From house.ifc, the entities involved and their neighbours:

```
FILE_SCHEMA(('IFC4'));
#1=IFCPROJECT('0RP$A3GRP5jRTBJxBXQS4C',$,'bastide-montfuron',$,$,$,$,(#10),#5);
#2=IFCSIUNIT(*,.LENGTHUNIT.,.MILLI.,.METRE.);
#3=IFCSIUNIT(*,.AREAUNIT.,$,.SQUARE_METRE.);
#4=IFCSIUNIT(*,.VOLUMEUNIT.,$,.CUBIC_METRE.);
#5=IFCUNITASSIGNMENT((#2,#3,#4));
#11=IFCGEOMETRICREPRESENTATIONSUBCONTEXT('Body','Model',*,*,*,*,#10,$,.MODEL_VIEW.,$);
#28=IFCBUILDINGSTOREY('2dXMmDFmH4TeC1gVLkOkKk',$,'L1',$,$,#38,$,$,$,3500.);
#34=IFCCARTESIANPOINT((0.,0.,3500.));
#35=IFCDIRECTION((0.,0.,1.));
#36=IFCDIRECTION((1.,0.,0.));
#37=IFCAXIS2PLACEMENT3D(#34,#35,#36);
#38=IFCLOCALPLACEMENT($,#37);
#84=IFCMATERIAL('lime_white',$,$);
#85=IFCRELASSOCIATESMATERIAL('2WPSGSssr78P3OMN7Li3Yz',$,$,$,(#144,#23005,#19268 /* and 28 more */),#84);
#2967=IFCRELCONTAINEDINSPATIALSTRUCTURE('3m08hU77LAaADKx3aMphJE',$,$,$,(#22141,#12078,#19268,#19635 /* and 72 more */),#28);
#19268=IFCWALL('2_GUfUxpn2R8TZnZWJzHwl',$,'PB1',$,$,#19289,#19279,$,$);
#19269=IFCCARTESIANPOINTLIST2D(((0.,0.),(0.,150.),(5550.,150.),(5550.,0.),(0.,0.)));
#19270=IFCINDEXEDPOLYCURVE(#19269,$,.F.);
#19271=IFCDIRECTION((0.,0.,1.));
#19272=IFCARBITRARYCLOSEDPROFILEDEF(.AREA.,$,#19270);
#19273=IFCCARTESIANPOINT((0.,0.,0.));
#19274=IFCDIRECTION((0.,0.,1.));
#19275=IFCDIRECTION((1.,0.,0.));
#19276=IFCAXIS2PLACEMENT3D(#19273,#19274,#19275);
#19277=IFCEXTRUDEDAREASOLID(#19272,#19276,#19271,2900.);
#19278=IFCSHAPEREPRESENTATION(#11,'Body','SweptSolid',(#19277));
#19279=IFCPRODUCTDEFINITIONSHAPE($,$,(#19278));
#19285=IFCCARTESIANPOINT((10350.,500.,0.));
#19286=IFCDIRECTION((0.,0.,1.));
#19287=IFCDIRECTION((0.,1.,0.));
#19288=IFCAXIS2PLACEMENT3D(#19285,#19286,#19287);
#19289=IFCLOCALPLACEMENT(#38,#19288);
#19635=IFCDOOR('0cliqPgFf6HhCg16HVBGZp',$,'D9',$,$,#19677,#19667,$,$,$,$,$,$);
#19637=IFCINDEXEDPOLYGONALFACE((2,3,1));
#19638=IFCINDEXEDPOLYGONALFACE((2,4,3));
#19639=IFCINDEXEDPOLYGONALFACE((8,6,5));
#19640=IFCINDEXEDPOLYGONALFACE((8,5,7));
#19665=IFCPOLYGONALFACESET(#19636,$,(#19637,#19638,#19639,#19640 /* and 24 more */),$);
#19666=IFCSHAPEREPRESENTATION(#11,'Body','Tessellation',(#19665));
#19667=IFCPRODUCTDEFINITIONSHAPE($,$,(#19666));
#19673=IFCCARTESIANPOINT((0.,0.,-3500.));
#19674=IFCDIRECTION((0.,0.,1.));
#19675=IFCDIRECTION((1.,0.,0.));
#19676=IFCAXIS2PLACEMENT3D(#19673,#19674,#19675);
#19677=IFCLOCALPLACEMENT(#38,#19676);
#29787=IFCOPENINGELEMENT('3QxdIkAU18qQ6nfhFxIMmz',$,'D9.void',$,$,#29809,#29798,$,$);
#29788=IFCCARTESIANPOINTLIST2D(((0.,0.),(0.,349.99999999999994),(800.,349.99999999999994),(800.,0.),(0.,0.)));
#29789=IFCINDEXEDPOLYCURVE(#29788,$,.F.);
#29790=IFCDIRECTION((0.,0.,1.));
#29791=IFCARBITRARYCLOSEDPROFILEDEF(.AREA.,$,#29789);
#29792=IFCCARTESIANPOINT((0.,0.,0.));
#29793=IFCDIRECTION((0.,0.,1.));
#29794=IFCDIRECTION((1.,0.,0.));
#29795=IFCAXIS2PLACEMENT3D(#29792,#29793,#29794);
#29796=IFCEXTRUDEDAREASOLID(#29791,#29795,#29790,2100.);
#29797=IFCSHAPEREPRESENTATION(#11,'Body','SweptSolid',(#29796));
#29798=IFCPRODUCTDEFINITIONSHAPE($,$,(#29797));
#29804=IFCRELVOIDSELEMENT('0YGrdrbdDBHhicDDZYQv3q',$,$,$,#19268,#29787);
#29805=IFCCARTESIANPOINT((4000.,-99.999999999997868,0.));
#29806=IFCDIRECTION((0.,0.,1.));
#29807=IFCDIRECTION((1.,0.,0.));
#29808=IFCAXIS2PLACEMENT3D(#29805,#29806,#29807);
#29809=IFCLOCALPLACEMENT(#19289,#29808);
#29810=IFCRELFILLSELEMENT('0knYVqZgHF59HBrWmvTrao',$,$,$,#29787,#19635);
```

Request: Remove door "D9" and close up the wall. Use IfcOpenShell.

```python
import ifcopenshell
import ifcopenshell.api.feature
import ifcopenshell.api.root
import ifcopenshell.geom
import ifcopenshell.util.shape

model = ifcopenshell.open("house.ifc")
settings = ifcopenshell.geom.settings()


def volume(element):
    """Net volume in cubic metres, openings subtracted."""
    shape = ifcopenshell.geom.create_shape(settings, element)
    return ifcopenshell.util.shape.get_volume(shape.geometry)


door = model.by_guid("0cliqPgFf6HhCg16HVBGZp")
opening = door.FillsVoids[0].RelatingOpeningElement
wall = opening.VoidsElements[0].RelatingBuildingElement
before = volume(wall)

ifcopenshell.api.root.remove_product(model, product=door)
ifcopenshell.api.feature.remove_feature(model, feature=opening)

after = volume(wall)

print(f"wall volume {before:.3f} -> {after:.3f} m3")

model.write("house_updated.ifc")
```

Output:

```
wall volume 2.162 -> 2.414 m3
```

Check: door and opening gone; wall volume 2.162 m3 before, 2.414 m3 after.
